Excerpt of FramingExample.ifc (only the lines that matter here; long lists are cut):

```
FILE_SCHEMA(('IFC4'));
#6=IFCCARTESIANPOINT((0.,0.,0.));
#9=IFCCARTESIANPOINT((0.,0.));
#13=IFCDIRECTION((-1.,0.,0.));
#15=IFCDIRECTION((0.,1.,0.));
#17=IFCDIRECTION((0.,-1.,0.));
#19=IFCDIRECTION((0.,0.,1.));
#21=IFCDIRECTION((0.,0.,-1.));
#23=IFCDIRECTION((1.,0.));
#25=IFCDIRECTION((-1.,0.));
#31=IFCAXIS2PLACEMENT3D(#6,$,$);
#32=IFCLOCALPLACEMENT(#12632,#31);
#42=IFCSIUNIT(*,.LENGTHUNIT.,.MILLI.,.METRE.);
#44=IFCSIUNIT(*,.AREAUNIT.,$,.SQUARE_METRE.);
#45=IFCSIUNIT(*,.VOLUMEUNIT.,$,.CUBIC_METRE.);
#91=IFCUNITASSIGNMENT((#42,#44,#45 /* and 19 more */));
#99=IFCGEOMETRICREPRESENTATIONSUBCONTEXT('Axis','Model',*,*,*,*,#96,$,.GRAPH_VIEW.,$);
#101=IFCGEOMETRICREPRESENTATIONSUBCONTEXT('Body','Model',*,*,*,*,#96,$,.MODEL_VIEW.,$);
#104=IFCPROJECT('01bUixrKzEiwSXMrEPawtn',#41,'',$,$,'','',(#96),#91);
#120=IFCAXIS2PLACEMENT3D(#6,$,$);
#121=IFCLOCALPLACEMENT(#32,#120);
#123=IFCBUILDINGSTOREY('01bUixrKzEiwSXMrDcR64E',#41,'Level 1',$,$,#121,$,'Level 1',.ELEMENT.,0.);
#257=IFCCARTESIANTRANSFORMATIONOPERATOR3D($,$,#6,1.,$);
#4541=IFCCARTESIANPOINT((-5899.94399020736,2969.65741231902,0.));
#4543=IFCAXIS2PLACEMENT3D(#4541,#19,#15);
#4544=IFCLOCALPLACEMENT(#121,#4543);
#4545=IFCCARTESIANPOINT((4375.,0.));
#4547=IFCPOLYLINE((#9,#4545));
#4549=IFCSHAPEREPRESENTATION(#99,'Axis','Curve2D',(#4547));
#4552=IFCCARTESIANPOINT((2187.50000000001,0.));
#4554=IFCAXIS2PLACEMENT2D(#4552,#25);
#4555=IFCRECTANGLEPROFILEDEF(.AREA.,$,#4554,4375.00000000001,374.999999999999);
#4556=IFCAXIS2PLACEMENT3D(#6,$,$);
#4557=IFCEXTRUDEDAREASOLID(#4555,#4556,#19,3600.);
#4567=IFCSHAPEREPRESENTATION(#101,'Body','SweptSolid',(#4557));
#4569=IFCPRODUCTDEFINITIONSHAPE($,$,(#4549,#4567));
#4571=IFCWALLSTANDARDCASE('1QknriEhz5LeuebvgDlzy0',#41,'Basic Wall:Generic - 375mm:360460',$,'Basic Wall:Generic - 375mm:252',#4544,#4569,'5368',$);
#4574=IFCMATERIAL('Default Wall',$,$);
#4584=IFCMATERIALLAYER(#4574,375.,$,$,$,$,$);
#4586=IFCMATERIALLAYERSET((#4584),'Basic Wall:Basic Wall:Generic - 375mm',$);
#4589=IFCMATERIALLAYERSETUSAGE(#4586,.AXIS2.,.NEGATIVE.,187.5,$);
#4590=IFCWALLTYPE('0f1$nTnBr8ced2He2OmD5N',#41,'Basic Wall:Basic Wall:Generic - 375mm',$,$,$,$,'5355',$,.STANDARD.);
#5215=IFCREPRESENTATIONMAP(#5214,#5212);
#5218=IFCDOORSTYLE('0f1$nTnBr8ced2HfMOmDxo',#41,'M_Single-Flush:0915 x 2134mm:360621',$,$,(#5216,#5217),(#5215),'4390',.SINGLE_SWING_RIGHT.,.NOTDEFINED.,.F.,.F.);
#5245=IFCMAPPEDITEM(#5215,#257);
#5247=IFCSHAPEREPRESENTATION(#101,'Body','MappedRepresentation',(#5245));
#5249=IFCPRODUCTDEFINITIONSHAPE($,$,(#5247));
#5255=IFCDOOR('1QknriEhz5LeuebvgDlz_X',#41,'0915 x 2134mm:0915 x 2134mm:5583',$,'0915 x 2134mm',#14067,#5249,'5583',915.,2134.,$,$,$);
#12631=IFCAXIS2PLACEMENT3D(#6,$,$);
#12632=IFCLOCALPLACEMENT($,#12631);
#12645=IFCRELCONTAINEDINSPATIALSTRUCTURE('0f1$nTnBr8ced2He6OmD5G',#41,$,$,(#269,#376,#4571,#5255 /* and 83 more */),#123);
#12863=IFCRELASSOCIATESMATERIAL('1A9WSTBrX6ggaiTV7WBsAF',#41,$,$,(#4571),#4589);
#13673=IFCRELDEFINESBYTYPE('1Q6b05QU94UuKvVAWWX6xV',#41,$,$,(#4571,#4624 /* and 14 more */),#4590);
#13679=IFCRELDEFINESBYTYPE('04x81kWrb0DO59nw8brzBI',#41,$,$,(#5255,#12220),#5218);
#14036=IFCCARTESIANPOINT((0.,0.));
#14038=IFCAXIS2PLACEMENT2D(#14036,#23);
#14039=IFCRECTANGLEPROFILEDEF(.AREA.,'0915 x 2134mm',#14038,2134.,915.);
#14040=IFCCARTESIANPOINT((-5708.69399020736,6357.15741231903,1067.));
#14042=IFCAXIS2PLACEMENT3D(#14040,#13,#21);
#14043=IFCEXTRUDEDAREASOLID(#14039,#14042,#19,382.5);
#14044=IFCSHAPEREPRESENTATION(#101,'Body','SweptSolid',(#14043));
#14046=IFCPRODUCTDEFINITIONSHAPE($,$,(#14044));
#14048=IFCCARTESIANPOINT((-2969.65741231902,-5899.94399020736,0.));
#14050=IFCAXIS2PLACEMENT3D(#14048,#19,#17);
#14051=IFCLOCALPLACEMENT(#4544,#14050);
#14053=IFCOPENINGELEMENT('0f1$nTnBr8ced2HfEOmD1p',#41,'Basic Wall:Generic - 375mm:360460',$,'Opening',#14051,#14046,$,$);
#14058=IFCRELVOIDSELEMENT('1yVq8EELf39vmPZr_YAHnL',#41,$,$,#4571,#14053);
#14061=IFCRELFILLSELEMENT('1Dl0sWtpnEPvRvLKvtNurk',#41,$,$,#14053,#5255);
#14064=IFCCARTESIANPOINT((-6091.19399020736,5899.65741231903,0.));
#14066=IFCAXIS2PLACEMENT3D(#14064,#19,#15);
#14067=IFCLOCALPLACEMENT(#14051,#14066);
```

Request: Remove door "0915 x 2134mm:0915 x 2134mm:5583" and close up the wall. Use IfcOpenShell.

```python
import ifcopenshell
import ifcopenshell.api.feature
import ifcopenshell.api.root
import ifcopenshell.geom
import ifcopenshell.util.shape

model = ifcopenshell.open("FramingExample.ifc")
settings = ifcopenshell.geom.settings()


def volume(element):
    """Net volume in cubic metres, openings subtracted."""
    shape = ifcopenshell.geom.create_shape(settings, element)
    return ifcopenshell.util.shape.get_volume(shape.geometry)


door = model.by_guid("1QknriEhz5LeuebvgDlz_X")
opening = door.FillsVoids[0].RelatingOpeningElement
wall = opening.VoidsElements[0].RelatingBuildingElement
before = volume(wall)

ifcopenshell.api.root.remove_product(model, product=door)
ifcopenshell.api.feature.remove_feature(model, feature=opening)

after = volume(wall)

print(f"wall volume {before:.3f} -> {after:.3f} m3")

model.write("FramingExample-out.ifc")
```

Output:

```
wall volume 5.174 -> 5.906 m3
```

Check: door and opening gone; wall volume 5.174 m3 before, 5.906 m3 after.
